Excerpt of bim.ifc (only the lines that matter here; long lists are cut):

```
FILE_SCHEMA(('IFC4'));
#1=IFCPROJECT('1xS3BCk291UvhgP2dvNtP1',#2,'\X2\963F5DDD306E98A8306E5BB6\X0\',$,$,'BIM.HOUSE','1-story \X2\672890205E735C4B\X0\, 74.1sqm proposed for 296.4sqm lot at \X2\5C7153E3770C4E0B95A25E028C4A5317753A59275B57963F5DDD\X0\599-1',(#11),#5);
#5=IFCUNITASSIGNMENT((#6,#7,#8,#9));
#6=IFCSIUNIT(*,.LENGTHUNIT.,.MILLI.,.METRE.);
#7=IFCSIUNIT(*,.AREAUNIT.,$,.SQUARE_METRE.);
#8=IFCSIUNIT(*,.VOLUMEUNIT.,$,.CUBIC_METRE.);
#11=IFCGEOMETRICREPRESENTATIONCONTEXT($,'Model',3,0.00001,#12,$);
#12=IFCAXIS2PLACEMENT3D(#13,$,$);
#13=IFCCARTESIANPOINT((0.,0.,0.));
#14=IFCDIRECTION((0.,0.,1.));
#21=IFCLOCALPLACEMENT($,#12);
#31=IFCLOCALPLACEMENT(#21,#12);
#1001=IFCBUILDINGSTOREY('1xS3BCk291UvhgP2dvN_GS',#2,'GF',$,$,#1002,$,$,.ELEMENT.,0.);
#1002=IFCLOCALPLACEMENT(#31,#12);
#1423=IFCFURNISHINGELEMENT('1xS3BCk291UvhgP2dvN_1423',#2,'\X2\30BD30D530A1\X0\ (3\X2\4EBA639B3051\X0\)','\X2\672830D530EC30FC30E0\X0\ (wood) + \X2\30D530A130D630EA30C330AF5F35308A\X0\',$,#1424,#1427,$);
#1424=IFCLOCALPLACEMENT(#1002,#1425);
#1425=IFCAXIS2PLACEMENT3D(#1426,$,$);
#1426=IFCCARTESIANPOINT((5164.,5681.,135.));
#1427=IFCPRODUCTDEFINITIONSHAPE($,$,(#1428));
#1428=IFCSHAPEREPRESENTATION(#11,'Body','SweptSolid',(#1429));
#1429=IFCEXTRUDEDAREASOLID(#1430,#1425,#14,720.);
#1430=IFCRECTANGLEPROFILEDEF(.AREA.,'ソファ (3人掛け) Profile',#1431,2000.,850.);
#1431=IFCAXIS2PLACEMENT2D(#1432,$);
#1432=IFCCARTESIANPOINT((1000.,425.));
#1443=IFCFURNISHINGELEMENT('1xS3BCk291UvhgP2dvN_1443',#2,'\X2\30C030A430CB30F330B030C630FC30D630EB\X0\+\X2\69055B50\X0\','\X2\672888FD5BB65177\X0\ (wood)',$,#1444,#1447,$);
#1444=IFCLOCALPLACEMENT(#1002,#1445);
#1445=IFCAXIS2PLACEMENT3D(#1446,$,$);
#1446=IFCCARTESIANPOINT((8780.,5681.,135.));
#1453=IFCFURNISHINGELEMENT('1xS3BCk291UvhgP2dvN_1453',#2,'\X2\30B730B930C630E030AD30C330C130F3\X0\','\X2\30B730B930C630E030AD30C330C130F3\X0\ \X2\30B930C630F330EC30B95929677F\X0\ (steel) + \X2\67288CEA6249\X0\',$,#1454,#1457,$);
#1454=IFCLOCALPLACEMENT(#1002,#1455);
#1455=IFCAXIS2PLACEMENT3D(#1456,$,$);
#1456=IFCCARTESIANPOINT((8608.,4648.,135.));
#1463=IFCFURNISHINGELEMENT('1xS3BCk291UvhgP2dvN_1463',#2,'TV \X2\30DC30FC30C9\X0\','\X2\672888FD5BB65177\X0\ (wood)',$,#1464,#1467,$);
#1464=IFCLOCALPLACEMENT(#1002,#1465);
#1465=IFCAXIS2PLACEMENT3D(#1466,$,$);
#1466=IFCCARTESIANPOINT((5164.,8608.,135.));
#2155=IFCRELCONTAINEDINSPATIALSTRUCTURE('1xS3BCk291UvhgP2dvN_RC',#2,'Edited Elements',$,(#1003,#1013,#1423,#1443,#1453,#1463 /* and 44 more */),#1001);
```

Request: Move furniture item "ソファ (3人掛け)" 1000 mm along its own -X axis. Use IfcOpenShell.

```python
import ifcopenshell
import ifcopenshell.api.geometry
import ifcopenshell.util.placement

model = ifcopenshell.open("bim.ifc")

item = model.by_id(1423)
matrix = ifcopenshell.util.placement.get_local_placement(item.ObjectPlacement)
matrix[:3, 3] -= matrix[:3, 0] * 1000.0
ifcopenshell.api.geometry.edit_object_placement(model, product=item, matrix=matrix, is_si=False)

print(ifcopenshell.util.placement.get_local_placement(item.ObjectPlacement).round(3) + 0.0)

model.write("bim_updated.ifc")
```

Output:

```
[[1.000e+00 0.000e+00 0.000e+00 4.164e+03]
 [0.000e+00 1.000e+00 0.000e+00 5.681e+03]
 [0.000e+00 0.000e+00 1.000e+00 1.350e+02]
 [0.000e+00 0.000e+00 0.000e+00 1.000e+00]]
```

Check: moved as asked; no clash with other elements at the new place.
